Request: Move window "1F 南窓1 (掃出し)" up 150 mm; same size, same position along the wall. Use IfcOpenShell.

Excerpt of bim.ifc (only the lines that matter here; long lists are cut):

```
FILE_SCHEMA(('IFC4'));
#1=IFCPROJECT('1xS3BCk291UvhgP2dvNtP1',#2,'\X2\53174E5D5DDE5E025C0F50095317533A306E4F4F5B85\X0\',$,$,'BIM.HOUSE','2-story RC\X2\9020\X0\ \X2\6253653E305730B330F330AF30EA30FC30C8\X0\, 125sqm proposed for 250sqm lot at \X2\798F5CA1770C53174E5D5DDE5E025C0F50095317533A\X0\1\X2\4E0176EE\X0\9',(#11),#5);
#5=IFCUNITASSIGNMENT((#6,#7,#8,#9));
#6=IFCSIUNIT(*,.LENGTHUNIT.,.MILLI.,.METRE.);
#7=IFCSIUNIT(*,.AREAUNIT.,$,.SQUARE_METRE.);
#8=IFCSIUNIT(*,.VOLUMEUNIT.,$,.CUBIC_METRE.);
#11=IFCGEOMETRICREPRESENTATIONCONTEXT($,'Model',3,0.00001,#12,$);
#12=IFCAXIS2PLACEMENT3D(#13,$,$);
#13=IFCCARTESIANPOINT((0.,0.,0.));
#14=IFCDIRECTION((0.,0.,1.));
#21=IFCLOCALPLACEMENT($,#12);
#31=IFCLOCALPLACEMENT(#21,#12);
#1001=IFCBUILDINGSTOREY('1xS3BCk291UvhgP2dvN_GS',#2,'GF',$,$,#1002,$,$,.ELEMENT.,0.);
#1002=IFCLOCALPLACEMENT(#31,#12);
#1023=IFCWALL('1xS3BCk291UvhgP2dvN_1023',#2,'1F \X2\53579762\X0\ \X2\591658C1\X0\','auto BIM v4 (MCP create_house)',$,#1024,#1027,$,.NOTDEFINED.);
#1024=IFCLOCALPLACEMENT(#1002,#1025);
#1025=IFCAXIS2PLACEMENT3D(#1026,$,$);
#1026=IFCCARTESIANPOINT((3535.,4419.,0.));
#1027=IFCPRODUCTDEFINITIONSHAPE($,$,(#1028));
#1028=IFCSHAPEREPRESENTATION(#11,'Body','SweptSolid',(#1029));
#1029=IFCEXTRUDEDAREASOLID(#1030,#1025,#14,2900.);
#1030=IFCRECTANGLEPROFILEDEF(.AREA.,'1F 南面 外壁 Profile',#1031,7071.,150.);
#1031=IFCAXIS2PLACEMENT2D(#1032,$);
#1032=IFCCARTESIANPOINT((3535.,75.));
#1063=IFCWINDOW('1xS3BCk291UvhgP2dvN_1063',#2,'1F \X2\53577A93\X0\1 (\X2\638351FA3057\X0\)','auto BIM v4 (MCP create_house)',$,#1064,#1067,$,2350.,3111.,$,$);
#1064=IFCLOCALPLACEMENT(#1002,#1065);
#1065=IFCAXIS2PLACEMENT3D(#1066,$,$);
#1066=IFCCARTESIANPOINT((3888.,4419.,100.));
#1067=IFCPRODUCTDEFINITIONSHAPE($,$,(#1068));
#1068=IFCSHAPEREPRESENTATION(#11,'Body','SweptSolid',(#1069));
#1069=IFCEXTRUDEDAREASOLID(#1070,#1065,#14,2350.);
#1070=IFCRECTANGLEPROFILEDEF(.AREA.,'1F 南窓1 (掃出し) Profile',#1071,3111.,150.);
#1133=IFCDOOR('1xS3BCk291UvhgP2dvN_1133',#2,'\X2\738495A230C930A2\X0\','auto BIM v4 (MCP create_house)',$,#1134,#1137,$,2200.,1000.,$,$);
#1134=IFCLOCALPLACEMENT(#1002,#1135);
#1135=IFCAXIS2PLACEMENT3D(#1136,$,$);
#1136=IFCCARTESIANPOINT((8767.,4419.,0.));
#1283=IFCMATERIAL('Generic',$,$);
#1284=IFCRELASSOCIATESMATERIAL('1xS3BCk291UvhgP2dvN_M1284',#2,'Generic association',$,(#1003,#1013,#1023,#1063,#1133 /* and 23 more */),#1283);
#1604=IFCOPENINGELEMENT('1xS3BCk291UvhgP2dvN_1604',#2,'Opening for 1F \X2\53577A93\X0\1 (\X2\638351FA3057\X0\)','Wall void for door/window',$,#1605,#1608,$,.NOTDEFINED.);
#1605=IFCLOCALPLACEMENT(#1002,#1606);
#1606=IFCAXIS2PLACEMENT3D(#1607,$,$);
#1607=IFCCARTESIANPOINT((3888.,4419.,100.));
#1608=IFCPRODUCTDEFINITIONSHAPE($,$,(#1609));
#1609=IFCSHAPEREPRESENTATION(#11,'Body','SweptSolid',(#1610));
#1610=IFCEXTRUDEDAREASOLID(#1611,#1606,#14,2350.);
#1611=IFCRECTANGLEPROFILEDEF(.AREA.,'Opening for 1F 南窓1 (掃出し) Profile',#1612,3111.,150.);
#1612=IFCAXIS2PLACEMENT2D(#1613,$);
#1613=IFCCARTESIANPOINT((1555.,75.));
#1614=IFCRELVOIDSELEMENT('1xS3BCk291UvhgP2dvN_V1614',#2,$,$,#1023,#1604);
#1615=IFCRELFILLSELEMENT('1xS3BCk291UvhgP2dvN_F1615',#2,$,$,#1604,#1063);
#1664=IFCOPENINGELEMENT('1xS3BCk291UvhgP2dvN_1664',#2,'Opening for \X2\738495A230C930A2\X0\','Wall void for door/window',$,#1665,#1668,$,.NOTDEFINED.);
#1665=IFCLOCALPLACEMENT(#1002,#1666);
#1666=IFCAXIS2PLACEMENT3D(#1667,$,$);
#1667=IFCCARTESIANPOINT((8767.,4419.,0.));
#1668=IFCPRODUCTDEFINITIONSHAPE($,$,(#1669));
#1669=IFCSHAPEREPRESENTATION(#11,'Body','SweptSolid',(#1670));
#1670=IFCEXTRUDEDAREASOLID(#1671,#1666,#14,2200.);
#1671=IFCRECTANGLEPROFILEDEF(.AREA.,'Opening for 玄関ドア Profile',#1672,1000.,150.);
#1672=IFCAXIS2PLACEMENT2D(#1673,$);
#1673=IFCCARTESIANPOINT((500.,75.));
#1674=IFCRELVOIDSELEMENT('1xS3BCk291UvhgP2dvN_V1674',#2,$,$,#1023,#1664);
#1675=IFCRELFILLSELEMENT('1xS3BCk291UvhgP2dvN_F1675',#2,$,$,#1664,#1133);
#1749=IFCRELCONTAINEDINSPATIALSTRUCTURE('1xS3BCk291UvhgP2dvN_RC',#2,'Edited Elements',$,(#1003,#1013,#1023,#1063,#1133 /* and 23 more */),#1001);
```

```python
import numpy as np
import ifcopenshell
import ifcopenshell.api.geometry
import ifcopenshell.util.placement
import ifcopenshell.util.unit

model = ifcopenshell.open("bim.ifc")
unit_scale = ifcopenshell.util.unit.calculate_unit_scale(model)

window = model.by_guid("1xS3BCk291UvhgP2dvN_1063")
opening = window.FillsVoids[0].RelatingOpeningElement
dz = 0.15 / unit_scale

shift = np.array([0.0, 0.0, dz])
# The window is not placed relative to its opening, so move both.
for product in (opening, window):
    matrix = ifcopenshell.util.placement.get_local_placement(product.ObjectPlacement)
    matrix[:3, 3] += shift
    ifcopenshell.api.geometry.edit_object_placement(model, product=product, matrix=matrix, is_si=False)

print(f"moved by {dz * unit_scale:+.3f} m")

model.write("bim_edited.ifc")
```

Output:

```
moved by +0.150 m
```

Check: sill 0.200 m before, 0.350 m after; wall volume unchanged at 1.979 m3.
